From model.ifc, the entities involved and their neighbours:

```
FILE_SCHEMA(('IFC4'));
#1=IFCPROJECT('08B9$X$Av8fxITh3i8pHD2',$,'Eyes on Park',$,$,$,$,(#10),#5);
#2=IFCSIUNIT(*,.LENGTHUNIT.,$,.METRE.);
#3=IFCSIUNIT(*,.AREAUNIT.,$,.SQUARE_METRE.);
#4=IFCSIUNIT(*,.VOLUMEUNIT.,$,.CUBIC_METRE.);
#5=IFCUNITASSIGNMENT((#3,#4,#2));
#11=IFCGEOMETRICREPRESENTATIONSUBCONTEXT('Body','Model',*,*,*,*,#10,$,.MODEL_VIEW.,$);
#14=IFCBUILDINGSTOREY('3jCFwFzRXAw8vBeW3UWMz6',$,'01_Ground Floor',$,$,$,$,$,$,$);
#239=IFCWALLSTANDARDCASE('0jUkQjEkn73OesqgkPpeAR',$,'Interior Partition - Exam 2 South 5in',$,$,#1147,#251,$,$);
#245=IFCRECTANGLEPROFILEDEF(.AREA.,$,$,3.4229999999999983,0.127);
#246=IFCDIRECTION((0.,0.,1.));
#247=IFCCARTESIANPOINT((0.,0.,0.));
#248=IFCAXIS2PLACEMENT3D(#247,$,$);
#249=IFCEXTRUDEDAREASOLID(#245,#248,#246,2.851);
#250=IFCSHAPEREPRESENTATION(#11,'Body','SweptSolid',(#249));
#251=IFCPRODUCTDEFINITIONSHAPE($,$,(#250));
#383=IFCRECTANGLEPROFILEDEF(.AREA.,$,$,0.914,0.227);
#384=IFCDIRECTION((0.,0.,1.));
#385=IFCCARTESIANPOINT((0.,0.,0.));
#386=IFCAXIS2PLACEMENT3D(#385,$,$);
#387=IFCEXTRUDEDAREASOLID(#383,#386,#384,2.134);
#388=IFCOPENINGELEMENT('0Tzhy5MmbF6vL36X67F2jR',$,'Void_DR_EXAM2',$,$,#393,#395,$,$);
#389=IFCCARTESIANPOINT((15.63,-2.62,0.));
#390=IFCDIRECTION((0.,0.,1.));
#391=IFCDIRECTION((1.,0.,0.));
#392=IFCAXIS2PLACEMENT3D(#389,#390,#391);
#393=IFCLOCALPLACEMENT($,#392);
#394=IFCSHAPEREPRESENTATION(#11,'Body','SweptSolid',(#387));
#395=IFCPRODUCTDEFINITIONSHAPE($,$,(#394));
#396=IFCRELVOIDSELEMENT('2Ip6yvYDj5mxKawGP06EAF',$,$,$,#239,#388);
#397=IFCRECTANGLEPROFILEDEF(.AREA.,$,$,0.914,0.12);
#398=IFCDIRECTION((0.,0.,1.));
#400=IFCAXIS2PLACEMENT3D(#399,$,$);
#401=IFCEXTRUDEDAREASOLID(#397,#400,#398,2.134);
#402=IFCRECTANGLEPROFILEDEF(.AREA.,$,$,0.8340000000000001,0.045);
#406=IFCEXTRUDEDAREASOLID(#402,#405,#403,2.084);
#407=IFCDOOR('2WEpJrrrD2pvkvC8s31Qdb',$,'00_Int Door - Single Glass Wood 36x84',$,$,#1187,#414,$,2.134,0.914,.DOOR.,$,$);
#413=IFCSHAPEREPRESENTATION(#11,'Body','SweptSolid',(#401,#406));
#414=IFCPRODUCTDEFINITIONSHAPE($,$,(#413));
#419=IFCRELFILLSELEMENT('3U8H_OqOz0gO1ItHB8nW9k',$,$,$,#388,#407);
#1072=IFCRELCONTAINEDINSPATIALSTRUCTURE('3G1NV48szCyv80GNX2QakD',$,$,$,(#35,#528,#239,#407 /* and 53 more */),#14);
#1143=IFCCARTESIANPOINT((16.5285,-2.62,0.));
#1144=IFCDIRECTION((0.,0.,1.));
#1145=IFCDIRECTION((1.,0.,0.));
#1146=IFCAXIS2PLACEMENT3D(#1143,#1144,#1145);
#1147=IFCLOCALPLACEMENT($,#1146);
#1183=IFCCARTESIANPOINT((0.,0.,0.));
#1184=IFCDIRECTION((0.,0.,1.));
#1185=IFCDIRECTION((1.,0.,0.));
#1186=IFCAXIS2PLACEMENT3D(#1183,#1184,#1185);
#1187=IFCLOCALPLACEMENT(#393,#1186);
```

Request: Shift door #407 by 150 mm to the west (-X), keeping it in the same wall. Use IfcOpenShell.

```python
import ifcopenshell
import ifcopenshell.api.geometry
import ifcopenshell.util.placement
import ifcopenshell.util.unit

model = ifcopenshell.open("model.ifc")
unit_scale = ifcopenshell.util.unit.calculate_unit_scale(model)

door = model.by_id(407)
opening = door.FillsVoids[0].RelatingOpeningElement
wall = opening.VoidsElements[0].RelatingBuildingElement

wall_matrix = ifcopenshell.util.placement.get_local_placement(wall.ObjectPlacement)
shift = wall_matrix[:3, 0] * -0.15 / unit_scale
before = ifcopenshell.util.placement.get_local_placement(door.ObjectPlacement)[:3, 3].copy()

# The door is placed relative to its opening, so it follows when the opening moves.
matrix = ifcopenshell.util.placement.get_local_placement(opening.ObjectPlacement)
matrix[:3, 3] += shift
ifcopenshell.api.geometry.edit_object_placement(
    model, product=opening, matrix=matrix, is_si=False, should_transform_children=True
)

after = ifcopenshell.util.placement.get_local_placement(door.ObjectPlacement)[:3, 3]
print("door moved by", (after - before).round(3) + 0.0)

model.write("model_edited.ifc")
```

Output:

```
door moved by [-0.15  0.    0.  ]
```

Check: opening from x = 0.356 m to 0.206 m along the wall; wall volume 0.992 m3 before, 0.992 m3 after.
